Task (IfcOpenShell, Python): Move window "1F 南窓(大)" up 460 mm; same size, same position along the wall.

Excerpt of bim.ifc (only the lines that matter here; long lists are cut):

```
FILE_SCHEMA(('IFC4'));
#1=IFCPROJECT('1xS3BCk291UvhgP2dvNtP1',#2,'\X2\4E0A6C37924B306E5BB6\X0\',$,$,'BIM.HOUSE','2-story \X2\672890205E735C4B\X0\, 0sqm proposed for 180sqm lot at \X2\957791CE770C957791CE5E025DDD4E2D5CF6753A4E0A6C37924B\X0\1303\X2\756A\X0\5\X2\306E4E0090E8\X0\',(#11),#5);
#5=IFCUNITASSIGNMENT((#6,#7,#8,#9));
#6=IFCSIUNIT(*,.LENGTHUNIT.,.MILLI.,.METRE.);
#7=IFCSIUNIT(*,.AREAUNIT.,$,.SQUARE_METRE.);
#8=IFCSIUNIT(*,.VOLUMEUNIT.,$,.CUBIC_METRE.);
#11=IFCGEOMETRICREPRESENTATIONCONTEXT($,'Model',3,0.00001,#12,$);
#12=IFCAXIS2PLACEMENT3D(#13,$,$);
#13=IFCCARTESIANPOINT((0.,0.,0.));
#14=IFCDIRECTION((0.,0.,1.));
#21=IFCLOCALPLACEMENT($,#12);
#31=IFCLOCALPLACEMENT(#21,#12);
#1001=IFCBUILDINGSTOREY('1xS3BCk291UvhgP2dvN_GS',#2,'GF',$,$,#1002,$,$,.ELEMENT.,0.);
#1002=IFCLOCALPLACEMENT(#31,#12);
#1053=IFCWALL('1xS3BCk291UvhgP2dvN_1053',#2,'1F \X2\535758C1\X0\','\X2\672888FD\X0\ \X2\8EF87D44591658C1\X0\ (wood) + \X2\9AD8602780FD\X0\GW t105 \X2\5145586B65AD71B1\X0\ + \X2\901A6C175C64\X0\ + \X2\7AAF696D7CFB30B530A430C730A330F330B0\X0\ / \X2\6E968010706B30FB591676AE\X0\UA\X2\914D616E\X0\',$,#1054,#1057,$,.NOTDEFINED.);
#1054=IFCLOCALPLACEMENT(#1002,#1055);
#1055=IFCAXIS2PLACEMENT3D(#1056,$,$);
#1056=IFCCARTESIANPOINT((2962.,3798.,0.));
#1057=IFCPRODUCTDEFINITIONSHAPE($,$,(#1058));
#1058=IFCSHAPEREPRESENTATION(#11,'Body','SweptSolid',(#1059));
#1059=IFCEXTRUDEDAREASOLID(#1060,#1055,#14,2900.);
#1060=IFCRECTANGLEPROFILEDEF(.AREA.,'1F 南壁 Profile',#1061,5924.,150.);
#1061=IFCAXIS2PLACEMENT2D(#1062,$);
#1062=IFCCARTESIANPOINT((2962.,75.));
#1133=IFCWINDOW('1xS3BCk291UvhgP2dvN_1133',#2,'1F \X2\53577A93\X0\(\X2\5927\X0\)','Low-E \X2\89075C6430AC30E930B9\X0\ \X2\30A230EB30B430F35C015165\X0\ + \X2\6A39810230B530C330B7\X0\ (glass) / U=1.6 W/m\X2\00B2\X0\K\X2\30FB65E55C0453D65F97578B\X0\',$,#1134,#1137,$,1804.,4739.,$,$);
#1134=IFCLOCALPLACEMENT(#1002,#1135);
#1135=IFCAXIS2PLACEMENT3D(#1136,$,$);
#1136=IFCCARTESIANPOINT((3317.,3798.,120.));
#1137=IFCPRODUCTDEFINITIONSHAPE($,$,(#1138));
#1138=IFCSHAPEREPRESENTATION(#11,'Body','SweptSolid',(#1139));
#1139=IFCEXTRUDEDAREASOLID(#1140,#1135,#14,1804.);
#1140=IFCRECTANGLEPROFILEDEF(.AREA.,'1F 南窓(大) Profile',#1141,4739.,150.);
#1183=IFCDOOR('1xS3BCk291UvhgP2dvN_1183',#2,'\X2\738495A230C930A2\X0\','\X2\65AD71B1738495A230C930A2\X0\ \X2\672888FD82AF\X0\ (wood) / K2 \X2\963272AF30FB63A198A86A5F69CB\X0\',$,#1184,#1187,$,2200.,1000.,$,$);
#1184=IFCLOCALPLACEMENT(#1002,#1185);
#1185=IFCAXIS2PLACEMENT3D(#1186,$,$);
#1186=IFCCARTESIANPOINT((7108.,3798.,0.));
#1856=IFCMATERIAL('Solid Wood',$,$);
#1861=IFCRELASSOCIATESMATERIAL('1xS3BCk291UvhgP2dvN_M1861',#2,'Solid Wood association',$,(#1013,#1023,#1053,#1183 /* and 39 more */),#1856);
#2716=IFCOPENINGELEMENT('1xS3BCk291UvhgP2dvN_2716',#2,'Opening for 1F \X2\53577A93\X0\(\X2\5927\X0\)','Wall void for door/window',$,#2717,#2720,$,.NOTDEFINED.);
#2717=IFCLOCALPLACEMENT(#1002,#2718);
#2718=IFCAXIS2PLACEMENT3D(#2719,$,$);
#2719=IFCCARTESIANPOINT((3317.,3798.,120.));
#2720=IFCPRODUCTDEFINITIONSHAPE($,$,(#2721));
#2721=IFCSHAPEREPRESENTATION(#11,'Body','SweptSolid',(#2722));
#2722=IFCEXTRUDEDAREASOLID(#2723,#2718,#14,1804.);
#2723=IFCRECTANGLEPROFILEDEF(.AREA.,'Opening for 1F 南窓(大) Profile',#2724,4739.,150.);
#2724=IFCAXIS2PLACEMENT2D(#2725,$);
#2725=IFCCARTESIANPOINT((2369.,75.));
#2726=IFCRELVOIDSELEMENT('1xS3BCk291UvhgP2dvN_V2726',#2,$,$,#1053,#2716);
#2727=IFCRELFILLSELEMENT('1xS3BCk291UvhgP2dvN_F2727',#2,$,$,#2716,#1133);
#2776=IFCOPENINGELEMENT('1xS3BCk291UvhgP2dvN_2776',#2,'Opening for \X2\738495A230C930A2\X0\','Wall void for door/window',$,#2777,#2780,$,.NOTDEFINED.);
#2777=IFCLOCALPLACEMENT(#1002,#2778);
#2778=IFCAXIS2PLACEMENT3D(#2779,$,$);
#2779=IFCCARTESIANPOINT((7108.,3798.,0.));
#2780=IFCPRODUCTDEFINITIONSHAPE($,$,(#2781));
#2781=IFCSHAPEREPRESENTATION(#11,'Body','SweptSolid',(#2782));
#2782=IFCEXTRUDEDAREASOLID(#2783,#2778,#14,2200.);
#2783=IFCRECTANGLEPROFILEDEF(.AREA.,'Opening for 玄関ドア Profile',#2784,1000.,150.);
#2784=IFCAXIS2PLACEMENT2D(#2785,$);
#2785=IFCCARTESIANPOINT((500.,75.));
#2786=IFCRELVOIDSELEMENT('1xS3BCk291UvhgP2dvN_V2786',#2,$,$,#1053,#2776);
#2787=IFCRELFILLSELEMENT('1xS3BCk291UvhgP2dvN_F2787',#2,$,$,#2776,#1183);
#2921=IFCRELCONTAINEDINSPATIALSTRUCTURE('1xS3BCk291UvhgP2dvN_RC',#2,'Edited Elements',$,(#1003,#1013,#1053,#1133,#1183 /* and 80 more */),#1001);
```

```python
import numpy as np
import ifcopenshell
import ifcopenshell.api.geometry
import ifcopenshell.util.placement
import ifcopenshell.util.unit

model = ifcopenshell.open("bim.ifc")
unit_scale = ifcopenshell.util.unit.calculate_unit_scale(model)

window = model.by_id(1133)
opening = window.FillsVoids[0].RelatingOpeningElement
dz = 460.0

shift = np.array([0.0, 0.0, dz])
# The window is not placed relative to its opening, so move both.
for product in (opening, window):
    matrix = ifcopenshell.util.placement.get_local_placement(product.ObjectPlacement)
    matrix[:3, 3] += shift
    ifcopenshell.api.geometry.edit_object_placement(model, product=product, matrix=matrix, is_si=False)

print(f"moved by {dz * unit_scale:+.3f} m")

model.write("bim_rev.ifc")
```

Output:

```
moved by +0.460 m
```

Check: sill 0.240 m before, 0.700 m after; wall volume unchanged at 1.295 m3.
